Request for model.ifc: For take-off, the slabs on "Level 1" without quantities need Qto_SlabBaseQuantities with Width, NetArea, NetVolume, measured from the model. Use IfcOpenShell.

First a look at what the model holds.

```python
import ifcopenshell
import ifcopenshell.util.element
import ifcopenshell.util.unit

model = ifcopenshell.open("model.ifc")
print(model.schema)
for unit_type in ("LENGTHUNIT", "AREAUNIT", "VOLUMEUNIT"):
    print(unit_type, ifcopenshell.util.unit.calculate_unit_scale(model, unit_type))
storey = next(s for s in model.by_type("IfcBuildingStorey") if s.Name == "Level 1")
slabs = [e for e in ifcopenshell.util.element.get_decomposition(storey) if e.is_a("IfcSlab")]
for e in sorted(slabs, key=lambda e: e.id()):
    print(e.id(), e.is_a(), e.Name, list(ifcopenshell.util.element.get_psets(e, qtos_only=True)), sep=" | ")
```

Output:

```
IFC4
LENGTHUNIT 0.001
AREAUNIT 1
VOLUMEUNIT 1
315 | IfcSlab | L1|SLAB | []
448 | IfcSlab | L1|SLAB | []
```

```python
import ifcopenshell
import ifcopenshell.api.pset
import ifcopenshell.geom
import ifcopenshell.util.element
import ifcopenshell.util.shape
import ifcopenshell.util.unit

model = ifcopenshell.open("model.ifc")
unit_scale = ifcopenshell.util.unit.calculate_unit_scale(model)
area_scale = ifcopenshell.util.unit.calculate_unit_scale(model, "AREAUNIT")
volume_scale = ifcopenshell.util.unit.calculate_unit_scale(model, "VOLUMEUNIT")
settings = ifcopenshell.geom.settings()

storey = next(s for s in model.by_type("IfcBuildingStorey") if s.Name == "Level 1")
slabs = [e for e in ifcopenshell.util.element.get_decomposition(storey) if e.is_a("IfcSlab")]

for e in sorted(slabs, key=lambda e: e.id()):
    if ifcopenshell.util.element.get_psets(e, qtos_only=True, should_inherit=False):
        continue
    # Geometry comes back in metres, in the element's own axes.
    shape = ifcopenshell.geom.create_shape(settings, e)
    values = {
        "Width": ifcopenshell.util.shape.get_z(shape.geometry) / unit_scale,
        "NetArea": ifcopenshell.util.shape.get_footprint_area(shape.geometry) / area_scale,
        "NetVolume": ifcopenshell.util.shape.get_volume(shape.geometry) / volume_scale,
    }
    qto = ifcopenshell.api.pset.add_qto(model, product=e, name="Qto_SlabBaseQuantities")
    ifcopenshell.api.pset.edit_qto(model, qto=qto, properties=values)
    print(e.id(), {k: round(v, 3) for k, v in values.items()})

model.write("model_edited.ifc")
```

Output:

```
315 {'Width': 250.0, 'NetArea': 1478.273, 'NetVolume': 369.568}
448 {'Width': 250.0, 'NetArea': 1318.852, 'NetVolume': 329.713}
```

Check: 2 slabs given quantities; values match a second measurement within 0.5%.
